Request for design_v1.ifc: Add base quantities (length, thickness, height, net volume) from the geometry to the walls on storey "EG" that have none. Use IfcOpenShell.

First a look at what the model holds.

```python
import ifcopenshell
import ifcopenshell.util.element
import ifcopenshell.util.unit

model = ifcopenshell.open("design_v1.ifc")
print(model.schema)
for unit_type in ("LENGTHUNIT", "AREAUNIT", "VOLUMEUNIT"):
    print(unit_type, ifcopenshell.util.unit.calculate_unit_scale(model, unit_type))
storey = next(s for s in model.by_type("IfcBuildingStorey") if s.Name == "EG")
walls = [e for e in ifcopenshell.util.element.get_decomposition(storey) if e.is_a("IfcWall")]
for e in sorted(walls, key=lambda e: e.id()):
    print(e.id(), e.is_a(), e.Name, list(ifcopenshell.util.element.get_psets(e, qtos_only=True)), sep=" | ")
```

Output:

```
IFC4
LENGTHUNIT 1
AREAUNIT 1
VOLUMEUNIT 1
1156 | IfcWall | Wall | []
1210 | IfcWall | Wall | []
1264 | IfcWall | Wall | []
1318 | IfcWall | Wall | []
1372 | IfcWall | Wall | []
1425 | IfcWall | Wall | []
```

```python
import ifcopenshell
import ifcopenshell.api.pset
import ifcopenshell.geom
import ifcopenshell.util.element
import ifcopenshell.util.shape
import ifcopenshell.util.unit

model = ifcopenshell.open("design_v1.ifc")
unit_scale = ifcopenshell.util.unit.calculate_unit_scale(model)
volume_scale = ifcopenshell.util.unit.calculate_unit_scale(model, "VOLUMEUNIT")
settings = ifcopenshell.geom.settings()

storey = next(s for s in model.by_type("IfcBuildingStorey") if s.Name == "EG")
walls = [e for e in ifcopenshell.util.element.get_decomposition(storey) if e.is_a("IfcWall")]

for e in sorted(walls, key=lambda e: e.id()):
    if ifcopenshell.util.element.get_psets(e, qtos_only=True, should_inherit=False):
        continue
    # Geometry comes back in metres, in the element's own axes.
    shape = ifcopenshell.geom.create_shape(settings, e)
    values = {
        "Length": ifcopenshell.util.shape.get_x(shape.geometry) / unit_scale,
        "Width": ifcopenshell.util.shape.get_y(shape.geometry) / unit_scale,
        "Height": ifcopenshell.util.shape.get_z(shape.geometry) / unit_scale,
        "NetVolume": ifcopenshell.util.shape.get_volume(shape.geometry) / volume_scale,
    }
    qto = ifcopenshell.api.pset.add_qto(model, product=e, name="Qto_WallBaseQuantities")
    ifcopenshell.api.pset.edit_qto(model, qto=qto, properties=values)
    print(e.id(), {k: round(v, 3) for k, v in values.items()})

model.write("design_v1_edited.ifc")
```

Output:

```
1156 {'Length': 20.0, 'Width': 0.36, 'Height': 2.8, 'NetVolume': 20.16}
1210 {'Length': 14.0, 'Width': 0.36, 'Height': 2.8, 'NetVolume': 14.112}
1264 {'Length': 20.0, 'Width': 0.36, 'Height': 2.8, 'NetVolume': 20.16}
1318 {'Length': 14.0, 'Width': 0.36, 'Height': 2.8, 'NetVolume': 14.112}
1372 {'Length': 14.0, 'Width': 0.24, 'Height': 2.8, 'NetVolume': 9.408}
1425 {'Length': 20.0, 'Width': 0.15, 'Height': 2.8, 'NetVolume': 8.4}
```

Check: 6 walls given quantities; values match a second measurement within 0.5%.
